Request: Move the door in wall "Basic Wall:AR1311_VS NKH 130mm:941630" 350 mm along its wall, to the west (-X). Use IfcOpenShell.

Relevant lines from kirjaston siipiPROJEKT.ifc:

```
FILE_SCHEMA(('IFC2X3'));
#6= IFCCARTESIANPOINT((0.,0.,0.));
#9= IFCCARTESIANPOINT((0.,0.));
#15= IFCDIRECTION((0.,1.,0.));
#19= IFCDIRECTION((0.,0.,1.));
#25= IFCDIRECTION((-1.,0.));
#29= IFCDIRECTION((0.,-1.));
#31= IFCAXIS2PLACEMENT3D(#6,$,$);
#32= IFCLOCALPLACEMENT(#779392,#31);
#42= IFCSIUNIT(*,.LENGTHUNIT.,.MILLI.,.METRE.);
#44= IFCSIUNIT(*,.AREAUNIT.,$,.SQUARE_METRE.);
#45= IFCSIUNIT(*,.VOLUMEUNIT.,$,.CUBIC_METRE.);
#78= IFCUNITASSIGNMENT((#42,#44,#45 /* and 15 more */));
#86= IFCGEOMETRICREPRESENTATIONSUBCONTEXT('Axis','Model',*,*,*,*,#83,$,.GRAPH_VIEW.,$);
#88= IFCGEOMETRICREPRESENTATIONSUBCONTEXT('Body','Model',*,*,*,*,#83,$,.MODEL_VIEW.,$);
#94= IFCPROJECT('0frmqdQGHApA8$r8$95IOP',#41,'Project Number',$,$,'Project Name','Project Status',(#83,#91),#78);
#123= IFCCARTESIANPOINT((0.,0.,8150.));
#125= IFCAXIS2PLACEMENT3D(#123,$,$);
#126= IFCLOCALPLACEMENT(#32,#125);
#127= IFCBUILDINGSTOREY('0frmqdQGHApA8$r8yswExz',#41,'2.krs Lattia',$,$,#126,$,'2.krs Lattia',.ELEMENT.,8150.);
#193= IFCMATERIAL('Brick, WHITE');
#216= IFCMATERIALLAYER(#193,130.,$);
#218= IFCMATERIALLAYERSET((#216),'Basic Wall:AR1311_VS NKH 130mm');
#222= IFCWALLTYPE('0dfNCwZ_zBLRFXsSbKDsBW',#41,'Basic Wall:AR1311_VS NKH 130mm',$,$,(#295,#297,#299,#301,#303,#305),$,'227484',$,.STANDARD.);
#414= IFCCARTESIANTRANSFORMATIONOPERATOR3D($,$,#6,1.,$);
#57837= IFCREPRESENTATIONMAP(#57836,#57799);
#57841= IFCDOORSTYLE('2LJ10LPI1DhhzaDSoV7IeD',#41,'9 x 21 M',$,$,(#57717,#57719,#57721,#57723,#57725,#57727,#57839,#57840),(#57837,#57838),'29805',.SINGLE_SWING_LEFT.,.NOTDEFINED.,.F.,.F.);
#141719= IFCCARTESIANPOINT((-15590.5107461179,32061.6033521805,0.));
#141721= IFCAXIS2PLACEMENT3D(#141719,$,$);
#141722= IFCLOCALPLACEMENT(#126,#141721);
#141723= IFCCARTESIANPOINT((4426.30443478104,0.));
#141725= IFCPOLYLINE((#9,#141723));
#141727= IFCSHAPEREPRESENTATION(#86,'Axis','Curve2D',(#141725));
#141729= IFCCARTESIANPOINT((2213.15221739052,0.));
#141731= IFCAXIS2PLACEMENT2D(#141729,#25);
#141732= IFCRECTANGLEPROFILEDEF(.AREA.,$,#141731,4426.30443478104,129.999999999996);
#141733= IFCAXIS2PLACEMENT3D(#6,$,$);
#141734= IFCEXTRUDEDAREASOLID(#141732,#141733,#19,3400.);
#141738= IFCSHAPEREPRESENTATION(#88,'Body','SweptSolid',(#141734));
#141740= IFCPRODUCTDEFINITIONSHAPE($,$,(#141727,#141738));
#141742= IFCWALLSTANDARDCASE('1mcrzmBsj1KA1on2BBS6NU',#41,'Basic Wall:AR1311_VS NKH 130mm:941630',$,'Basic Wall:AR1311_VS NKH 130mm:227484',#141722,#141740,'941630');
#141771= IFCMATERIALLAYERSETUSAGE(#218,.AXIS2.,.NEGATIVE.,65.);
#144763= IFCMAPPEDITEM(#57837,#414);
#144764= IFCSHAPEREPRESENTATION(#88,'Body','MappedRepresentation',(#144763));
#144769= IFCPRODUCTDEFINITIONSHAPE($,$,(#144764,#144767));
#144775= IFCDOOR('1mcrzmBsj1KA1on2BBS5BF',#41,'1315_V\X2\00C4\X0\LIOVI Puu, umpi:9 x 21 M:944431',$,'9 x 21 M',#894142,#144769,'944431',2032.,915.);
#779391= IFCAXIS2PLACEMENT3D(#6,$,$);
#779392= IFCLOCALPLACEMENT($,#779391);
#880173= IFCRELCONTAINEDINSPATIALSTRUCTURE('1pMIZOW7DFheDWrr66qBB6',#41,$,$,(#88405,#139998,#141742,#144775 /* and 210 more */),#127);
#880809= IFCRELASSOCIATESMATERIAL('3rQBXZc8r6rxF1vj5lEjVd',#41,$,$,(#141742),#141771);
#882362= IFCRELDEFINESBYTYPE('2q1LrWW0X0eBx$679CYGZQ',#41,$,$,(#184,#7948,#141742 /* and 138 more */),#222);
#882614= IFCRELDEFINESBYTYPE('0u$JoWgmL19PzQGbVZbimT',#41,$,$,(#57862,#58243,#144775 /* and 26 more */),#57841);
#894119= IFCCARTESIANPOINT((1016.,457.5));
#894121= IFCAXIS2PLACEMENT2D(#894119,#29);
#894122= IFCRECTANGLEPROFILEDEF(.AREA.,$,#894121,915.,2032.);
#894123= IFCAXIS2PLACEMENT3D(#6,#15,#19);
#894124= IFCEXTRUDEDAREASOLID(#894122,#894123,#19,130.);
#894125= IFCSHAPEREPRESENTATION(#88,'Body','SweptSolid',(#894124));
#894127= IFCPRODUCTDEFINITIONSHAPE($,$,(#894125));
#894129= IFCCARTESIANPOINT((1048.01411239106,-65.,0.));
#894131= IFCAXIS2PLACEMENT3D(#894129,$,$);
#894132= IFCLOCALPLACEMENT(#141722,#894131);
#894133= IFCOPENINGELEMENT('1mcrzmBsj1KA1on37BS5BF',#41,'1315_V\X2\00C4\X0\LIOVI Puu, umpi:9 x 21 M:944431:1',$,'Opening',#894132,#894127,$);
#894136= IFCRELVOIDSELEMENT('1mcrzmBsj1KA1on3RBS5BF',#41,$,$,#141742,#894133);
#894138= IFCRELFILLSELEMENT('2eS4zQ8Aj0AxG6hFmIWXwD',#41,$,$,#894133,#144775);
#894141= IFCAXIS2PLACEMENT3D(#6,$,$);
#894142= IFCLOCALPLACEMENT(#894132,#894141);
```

```python
import ifcopenshell
import ifcopenshell.api.geometry
import ifcopenshell.util.placement

model = ifcopenshell.open("kirjaston siipiPROJEKT.ifc")

door = model.by_guid("1mcrzmBsj1KA1on2BBS5BF")
opening = door.FillsVoids[0].RelatingOpeningElement
wall = opening.VoidsElements[0].RelatingBuildingElement

wall_matrix = ifcopenshell.util.placement.get_local_placement(wall.ObjectPlacement)
shift = wall_matrix[:3, 0] * -350.0
before = ifcopenshell.util.placement.get_local_placement(door.ObjectPlacement)[:3, 3].copy()

# The door is placed relative to its opening, so it follows when the opening moves.
matrix = ifcopenshell.util.placement.get_local_placement(opening.ObjectPlacement)
matrix[:3, 3] += shift
ifcopenshell.api.geometry.edit_object_placement(
    model, product=opening, matrix=matrix, is_si=False, should_transform_children=True
)

after = ifcopenshell.util.placement.get_local_placement(door.ObjectPlacement)[:3, 3]
print("door moved by", (after - before).round(3) + 0.0)

model.write("kirjaston siipiPROJEKT_rev.ifc")
```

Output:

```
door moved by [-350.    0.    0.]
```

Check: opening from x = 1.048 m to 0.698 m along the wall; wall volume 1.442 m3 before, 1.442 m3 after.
